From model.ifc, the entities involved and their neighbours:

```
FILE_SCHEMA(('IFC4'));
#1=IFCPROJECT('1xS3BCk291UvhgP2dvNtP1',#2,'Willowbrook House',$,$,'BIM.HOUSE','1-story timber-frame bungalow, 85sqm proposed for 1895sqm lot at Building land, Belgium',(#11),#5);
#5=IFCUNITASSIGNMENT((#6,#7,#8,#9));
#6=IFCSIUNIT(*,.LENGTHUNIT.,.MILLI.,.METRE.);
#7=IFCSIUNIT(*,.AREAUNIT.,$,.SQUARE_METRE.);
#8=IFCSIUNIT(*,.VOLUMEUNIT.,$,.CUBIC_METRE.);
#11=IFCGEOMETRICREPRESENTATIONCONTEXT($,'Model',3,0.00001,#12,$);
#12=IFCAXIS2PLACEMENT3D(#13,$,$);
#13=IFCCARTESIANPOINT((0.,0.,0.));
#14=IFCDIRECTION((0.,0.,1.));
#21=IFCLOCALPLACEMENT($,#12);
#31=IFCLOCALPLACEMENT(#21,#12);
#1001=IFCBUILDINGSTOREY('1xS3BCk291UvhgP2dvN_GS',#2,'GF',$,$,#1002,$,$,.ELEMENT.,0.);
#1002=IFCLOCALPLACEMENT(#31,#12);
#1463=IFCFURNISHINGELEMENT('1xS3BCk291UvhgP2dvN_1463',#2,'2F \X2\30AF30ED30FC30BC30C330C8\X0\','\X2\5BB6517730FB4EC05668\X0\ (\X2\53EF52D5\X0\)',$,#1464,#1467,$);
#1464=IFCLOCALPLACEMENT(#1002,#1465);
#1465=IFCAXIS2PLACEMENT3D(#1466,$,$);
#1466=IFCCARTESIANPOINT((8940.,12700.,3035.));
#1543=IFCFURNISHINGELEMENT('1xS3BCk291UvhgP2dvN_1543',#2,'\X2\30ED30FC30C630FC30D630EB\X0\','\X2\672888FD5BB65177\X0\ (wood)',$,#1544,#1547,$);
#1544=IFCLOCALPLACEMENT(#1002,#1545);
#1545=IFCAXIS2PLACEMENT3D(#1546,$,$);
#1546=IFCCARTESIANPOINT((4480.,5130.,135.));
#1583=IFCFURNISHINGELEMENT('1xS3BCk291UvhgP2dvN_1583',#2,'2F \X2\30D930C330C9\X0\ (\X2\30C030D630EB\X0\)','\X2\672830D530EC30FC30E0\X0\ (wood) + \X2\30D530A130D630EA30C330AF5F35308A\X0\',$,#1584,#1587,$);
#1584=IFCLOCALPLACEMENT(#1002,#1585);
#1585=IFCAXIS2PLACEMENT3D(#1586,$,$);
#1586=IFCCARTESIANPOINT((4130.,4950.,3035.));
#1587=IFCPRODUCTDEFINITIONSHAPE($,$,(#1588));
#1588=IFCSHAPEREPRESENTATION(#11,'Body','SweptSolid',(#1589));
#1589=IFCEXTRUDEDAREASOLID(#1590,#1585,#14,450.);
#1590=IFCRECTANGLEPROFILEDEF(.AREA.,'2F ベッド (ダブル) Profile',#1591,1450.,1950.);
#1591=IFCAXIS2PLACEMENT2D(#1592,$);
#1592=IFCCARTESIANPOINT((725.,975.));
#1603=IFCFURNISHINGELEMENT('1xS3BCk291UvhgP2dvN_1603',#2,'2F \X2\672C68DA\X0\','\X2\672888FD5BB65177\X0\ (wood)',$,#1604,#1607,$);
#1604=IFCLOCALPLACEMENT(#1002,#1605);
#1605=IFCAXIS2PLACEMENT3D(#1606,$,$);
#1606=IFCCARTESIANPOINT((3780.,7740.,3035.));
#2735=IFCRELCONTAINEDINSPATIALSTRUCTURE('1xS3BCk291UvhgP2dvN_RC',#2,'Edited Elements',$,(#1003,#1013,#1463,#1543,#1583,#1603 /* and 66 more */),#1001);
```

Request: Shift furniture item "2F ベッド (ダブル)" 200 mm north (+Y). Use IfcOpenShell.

```python
import ifcopenshell
import ifcopenshell.api.geometry
import ifcopenshell.util.placement

model = ifcopenshell.open("model.ifc")

item = model.by_id(1583)
matrix = ifcopenshell.util.placement.get_local_placement(item.ObjectPlacement)
matrix[1, 3] += 200.0
ifcopenshell.api.geometry.edit_object_placement(model, product=item, matrix=matrix, is_si=False)

print(ifcopenshell.util.placement.get_local_placement(item.ObjectPlacement).round(3) + 0.0)

model.write("model_rev.ifc")
```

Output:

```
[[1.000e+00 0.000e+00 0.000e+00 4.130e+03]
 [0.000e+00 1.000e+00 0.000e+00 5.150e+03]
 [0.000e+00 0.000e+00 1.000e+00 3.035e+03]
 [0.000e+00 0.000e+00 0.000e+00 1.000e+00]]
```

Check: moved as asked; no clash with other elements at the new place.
